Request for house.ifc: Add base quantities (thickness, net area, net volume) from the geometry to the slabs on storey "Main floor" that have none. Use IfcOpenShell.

First a look at what the model holds.

```python
import ifcopenshell
import ifcopenshell.util.element
import ifcopenshell.util.unit

model = ifcopenshell.open("house.ifc")
print(model.schema)
for unit_type in ("LENGTHUNIT", "AREAUNIT", "VOLUMEUNIT"):
    print(unit_type, ifcopenshell.util.unit.calculate_unit_scale(model, unit_type))
storey = next(s for s in model.by_type("IfcBuildingStorey") if s.Name == "Main floor")
slabs = [e for e in ifcopenshell.util.element.get_decomposition(storey) if e.is_a("IfcSlab")]
for e in sorted(slabs, key=lambda e: e.id()):
    print(e.id(), e.is_a(), e.Name, list(ifcopenshell.util.element.get_psets(e, qtos_only=True)), sep=" | ")
```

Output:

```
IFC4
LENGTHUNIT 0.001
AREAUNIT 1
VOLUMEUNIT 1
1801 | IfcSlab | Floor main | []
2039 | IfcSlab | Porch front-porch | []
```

```python
import ifcopenshell
import ifcopenshell.api.pset
import ifcopenshell.geom
import ifcopenshell.util.element
import ifcopenshell.util.shape
import ifcopenshell.util.unit

model = ifcopenshell.open("house.ifc")
unit_scale = ifcopenshell.util.unit.calculate_unit_scale(model)
area_scale = ifcopenshell.util.unit.calculate_unit_scale(model, "AREAUNIT")
volume_scale = ifcopenshell.util.unit.calculate_unit_scale(model, "VOLUMEUNIT")
settings = ifcopenshell.geom.settings()

storey = next(s for s in model.by_type("IfcBuildingStorey") if s.Name == "Main floor")
slabs = [e for e in ifcopenshell.util.element.get_decomposition(storey) if e.is_a("IfcSlab")]

for e in sorted(slabs, key=lambda e: e.id()):
    if ifcopenshell.util.element.get_psets(e, qtos_only=True, should_inherit=False):
        continue
    # Geometry comes back in metres, in the element's own axes.
    shape = ifcopenshell.geom.create_shape(settings, e)
    values = {
        "Width": ifcopenshell.util.shape.get_z(shape.geometry) / unit_scale,
        "NetArea": ifcopenshell.util.shape.get_footprint_area(shape.geometry) / area_scale,
        "NetVolume": ifcopenshell.util.shape.get_volume(shape.geometry) / volume_scale,
    }
    qto = ifcopenshell.api.pset.add_qto(model, product=e, name="Qto_SlabBaseQuantities")
    ifcopenshell.api.pset.edit_qto(model, qto=qto, properties=values)
    print(e.id(), {k: round(v, 3) for k, v in values.items()})

model.write("house_v2.ifc")
```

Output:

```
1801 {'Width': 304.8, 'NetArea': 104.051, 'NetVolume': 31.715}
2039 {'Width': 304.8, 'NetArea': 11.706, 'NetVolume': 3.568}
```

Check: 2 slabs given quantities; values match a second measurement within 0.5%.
